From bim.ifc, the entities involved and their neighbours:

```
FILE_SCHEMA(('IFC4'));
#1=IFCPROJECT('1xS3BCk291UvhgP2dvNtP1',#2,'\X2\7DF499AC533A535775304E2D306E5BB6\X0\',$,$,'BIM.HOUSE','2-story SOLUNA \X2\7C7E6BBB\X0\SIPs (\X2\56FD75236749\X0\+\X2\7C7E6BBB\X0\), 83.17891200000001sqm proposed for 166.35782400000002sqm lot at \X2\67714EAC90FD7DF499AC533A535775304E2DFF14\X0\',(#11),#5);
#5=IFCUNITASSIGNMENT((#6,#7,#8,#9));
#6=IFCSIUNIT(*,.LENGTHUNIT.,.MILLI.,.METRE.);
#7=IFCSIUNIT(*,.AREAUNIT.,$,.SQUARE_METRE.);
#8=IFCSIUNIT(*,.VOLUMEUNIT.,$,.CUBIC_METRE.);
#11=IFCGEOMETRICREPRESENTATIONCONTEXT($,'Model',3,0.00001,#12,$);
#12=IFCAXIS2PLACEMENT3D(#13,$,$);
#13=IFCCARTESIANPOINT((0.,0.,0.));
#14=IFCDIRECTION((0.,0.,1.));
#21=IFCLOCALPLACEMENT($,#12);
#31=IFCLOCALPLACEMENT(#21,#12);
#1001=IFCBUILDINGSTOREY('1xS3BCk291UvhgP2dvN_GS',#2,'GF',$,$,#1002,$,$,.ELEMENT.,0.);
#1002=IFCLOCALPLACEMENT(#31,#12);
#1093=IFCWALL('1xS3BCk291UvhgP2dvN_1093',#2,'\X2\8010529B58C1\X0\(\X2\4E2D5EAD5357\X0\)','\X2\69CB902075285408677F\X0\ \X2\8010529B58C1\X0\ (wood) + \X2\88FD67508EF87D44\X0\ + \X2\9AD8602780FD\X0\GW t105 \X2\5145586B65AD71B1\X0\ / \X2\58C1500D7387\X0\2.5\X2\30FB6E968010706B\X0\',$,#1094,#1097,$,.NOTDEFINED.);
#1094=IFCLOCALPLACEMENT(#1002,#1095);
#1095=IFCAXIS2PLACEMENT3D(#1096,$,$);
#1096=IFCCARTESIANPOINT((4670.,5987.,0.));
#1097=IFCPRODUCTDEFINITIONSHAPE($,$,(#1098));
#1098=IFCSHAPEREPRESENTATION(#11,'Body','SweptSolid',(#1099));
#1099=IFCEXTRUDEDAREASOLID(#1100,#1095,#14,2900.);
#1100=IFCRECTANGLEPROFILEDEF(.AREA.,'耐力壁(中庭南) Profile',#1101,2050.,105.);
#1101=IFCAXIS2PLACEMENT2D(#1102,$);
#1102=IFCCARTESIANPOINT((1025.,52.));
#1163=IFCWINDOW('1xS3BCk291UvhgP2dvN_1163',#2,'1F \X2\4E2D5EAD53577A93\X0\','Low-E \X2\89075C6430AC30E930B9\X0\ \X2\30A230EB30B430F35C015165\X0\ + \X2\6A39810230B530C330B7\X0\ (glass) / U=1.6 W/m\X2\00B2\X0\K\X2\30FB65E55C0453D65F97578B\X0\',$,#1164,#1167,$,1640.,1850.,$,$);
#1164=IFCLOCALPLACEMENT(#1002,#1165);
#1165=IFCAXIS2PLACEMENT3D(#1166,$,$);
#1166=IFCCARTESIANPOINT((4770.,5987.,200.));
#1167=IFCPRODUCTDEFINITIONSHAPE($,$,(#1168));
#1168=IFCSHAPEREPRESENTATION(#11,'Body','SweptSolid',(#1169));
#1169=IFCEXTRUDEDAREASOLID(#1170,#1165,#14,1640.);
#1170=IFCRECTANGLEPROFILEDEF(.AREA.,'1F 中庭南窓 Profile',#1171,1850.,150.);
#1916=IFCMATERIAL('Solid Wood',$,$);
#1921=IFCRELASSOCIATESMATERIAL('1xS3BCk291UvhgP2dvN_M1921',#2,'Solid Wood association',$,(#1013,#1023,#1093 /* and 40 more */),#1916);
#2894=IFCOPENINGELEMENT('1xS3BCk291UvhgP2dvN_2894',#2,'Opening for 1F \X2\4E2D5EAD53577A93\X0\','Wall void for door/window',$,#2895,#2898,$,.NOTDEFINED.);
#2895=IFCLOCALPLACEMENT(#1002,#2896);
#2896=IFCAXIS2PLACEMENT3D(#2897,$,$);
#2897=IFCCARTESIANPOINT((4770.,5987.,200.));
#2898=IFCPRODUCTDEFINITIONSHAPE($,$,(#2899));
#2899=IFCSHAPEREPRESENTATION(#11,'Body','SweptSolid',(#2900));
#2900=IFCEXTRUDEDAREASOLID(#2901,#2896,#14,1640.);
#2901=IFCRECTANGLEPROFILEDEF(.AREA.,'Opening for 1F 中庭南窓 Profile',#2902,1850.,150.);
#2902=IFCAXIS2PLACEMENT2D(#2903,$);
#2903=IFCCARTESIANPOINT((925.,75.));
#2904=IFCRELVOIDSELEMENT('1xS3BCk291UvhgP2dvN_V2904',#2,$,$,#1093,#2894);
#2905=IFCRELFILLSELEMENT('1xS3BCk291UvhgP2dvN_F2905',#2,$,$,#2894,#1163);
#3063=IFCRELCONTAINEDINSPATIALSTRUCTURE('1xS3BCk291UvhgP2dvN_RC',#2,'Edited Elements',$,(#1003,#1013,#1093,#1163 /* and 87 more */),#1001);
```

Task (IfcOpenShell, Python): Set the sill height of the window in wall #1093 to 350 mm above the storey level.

```python
import numpy as np
import ifcopenshell
import ifcopenshell.api.geometry
import ifcopenshell.geom
import ifcopenshell.util.element
import ifcopenshell.util.placement
import ifcopenshell.util.shape
import ifcopenshell.util.unit

model = ifcopenshell.open("bim.ifc")
unit_scale = ifcopenshell.util.unit.calculate_unit_scale(model)

window = model.by_guid("1xS3BCk291UvhgP2dvN_1163")
opening = window.FillsVoids[0].RelatingOpeningElement
storey = ifcopenshell.util.element.get_container(window, ifc_class="IfcBuildingStorey")
level = ifcopenshell.util.placement.get_local_placement(storey.ObjectPlacement)[2, 3]

# The opening's origin need not be at the sill, so measure its lowest point.
shape = ifcopenshell.geom.create_shape(ifcopenshell.geom.settings(), opening)
bottom = ifcopenshell.util.shape.get_shape_bottom_elevation(shape, shape.geometry) / unit_scale
dz = level + 0.35 / unit_scale - bottom

shift = np.array([0.0, 0.0, dz])
# The window is not placed relative to its opening, so move both.
for product in (opening, window):
    matrix = ifcopenshell.util.placement.get_local_placement(product.ObjectPlacement)
    matrix[:3, 3] += shift
    ifcopenshell.api.geometry.edit_object_placement(model, product=product, matrix=matrix, is_si=False)

print(f"moved by {dz * unit_scale:+.3f} m")

model.write("bim_rev.ifc")
```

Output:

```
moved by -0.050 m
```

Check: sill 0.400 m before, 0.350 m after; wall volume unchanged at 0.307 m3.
